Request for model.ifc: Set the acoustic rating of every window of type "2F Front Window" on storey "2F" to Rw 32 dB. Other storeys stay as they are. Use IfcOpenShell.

First a look at what the model holds.

```python
import ifcopenshell
import ifcopenshell.util.element

model = ifcopenshell.open("model.ifc")
print(model.schema)
storey = next(s for s in model.by_type("IfcBuildingStorey") if s.Name == "2F")
windows = [e for e in ifcopenshell.util.element.get_decomposition(storey) if e.is_a("IfcWindow")]
seen = {}
for e in windows:
    element_type = ifcopenshell.util.element.get_type(e)
    key = (element_type.Name if element_type != e and element_type else None, ifcopenshell.util.element.get_pset(e, "Pset_WindowCommon", "AcousticRating"))
    seen[key] = seen.get(key, 0) + 1
for (name, value), count in sorted(seen.items(), key=str):
    print(count, "x", name, "|", value)
```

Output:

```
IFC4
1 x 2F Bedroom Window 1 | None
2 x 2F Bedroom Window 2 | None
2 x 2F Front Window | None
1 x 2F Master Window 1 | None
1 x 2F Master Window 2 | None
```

```python
import ifcopenshell
import ifcopenshell.api.pset
import ifcopenshell.util.element

model = ifcopenshell.open("model.ifc")

storey = next(s for s in model.by_type("IfcBuildingStorey") if s.Name == "2F")
windows = [e for e in ifcopenshell.util.element.get_decomposition(storey) if e.is_a("IfcWindow")]

count = 0
for e in windows:
    element_type = ifcopenshell.util.element.get_type(e)
    if element_type in (None, e) or element_type.Name != "2F Front Window":
        continue
    # add_pset returns the element's existing set when there is one.
    pset = ifcopenshell.api.pset.add_pset(model, product=e, name="Pset_WindowCommon")
    ifcopenshell.api.pset.edit_pset(model, pset=pset, properties={"AcousticRating": "Rw 32 dB"})
    count += 1

print(count, "windows updated")

model.write("model_updated.ifc")
```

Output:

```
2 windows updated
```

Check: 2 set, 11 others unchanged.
